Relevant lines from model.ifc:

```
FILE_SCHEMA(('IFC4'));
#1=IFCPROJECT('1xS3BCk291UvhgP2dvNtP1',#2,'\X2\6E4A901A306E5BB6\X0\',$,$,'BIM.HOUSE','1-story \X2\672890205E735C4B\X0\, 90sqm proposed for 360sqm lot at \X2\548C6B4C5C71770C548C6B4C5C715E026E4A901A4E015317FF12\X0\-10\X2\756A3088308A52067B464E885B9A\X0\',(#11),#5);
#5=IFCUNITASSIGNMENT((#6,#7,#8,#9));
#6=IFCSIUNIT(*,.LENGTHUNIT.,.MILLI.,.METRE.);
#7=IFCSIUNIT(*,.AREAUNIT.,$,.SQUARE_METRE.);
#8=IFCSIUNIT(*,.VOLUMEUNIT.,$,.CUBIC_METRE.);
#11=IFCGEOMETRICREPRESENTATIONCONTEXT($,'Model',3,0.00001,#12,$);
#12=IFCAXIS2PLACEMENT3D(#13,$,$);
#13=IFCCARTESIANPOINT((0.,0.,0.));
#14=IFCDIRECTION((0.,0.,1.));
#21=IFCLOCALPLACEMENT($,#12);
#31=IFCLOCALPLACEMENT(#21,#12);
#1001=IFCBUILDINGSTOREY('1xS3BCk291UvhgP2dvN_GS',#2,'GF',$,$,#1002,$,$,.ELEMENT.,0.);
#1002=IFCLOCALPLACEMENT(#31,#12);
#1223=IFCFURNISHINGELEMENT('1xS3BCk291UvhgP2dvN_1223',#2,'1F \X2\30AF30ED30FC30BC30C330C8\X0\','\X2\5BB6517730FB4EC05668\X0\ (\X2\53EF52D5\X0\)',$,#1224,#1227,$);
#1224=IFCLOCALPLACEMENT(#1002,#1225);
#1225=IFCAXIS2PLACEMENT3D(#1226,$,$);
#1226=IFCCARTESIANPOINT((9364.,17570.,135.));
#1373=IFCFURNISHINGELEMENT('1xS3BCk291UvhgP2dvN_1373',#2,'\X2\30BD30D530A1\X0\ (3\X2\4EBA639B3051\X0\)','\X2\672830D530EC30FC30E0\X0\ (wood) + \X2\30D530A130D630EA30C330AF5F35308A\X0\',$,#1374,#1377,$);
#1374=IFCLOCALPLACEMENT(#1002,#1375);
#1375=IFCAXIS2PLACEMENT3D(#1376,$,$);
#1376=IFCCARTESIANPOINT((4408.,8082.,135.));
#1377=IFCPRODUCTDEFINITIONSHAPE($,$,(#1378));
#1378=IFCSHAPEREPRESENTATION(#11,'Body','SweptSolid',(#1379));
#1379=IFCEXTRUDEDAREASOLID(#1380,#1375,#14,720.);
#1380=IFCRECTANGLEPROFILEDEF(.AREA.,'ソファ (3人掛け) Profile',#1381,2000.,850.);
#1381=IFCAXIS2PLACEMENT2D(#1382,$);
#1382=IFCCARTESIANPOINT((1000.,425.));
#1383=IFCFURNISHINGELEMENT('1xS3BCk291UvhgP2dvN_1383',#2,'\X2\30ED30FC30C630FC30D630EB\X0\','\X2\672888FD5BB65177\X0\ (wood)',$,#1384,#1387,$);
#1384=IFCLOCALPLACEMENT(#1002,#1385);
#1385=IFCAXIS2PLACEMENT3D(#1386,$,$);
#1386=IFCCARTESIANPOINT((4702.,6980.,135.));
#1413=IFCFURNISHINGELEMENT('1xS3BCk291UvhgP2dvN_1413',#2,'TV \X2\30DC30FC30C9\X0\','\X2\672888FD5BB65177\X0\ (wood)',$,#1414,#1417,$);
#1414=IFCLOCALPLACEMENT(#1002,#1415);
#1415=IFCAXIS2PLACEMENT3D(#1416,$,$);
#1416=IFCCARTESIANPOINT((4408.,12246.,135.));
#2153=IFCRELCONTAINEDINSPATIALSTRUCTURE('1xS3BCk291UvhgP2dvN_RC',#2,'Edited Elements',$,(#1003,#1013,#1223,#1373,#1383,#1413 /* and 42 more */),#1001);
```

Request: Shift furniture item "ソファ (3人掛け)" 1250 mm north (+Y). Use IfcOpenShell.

```python
import ifcopenshell
import ifcopenshell.api.geometry
import ifcopenshell.util.placement
import ifcopenshell.util.unit

model = ifcopenshell.open("model.ifc")
unit_scale = ifcopenshell.util.unit.calculate_unit_scale(model)

item = model.by_id(1373)
matrix = ifcopenshell.util.placement.get_local_placement(item.ObjectPlacement)
matrix[1, 3] += 1.25 / unit_scale
ifcopenshell.api.geometry.edit_object_placement(model, product=item, matrix=matrix, is_si=False)

print(ifcopenshell.util.placement.get_local_placement(item.ObjectPlacement).round(3) + 0.0)

model.write("model_updated.ifc")
```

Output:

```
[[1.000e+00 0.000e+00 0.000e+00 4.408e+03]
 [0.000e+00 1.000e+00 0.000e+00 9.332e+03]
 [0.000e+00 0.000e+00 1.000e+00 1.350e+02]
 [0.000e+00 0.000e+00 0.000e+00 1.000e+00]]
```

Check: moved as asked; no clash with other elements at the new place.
